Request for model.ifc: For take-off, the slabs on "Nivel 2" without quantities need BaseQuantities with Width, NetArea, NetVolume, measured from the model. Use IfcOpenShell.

First a look at what the model holds.

```python
import ifcopenshell
import ifcopenshell.util.element
import ifcopenshell.util.unit

model = ifcopenshell.open("model.ifc")
print(model.schema)
for unit_type in ("LENGTHUNIT", "AREAUNIT", "VOLUMEUNIT"):
    print(unit_type, ifcopenshell.util.unit.calculate_unit_scale(model, unit_type))
storey = next(s for s in model.by_type("IfcBuildingStorey") if s.Name == "Nivel 2")
slabs = [e for e in ifcopenshell.util.element.get_decomposition(storey) if e.is_a("IfcSlab")]
for e in sorted(slabs, key=lambda e: e.id()):
    print(e.id(), e.is_a(), e.Name, list(ifcopenshell.util.element.get_psets(e, qtos_only=True)), sep=" | ")
```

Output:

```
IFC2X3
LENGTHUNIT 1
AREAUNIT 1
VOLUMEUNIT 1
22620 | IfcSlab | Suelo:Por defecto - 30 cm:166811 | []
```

```python
import ifcopenshell
import ifcopenshell.api.pset
import ifcopenshell.geom
import ifcopenshell.util.element
import ifcopenshell.util.shape
import ifcopenshell.util.unit

model = ifcopenshell.open("model.ifc")
unit_scale = ifcopenshell.util.unit.calculate_unit_scale(model)
area_scale = ifcopenshell.util.unit.calculate_unit_scale(model, "AREAUNIT")
volume_scale = ifcopenshell.util.unit.calculate_unit_scale(model, "VOLUMEUNIT")
settings = ifcopenshell.geom.settings()

storey = next(s for s in model.by_type("IfcBuildingStorey") if s.Name == "Nivel 2")
slabs = [e for e in ifcopenshell.util.element.get_decomposition(storey) if e.is_a("IfcSlab")]

for e in sorted(slabs, key=lambda e: e.id()):
    if ifcopenshell.util.element.get_psets(e, qtos_only=True, should_inherit=False):
        continue
    # Geometry comes back in metres, in the element's own axes.
    shape = ifcopenshell.geom.create_shape(settings, e)
    values = {
        "Width": ifcopenshell.util.shape.get_z(shape.geometry) / unit_scale,
        "NetArea": ifcopenshell.util.shape.get_footprint_area(shape.geometry) / area_scale,
        "NetVolume": ifcopenshell.util.shape.get_volume(shape.geometry) / volume_scale,
    }
    qto = ifcopenshell.api.pset.add_qto(model, product=e, name="BaseQuantities")
    ifcopenshell.api.pset.edit_qto(model, qto=qto, properties=values)
    print(e.id(), {k: round(v, 3) for k, v in values.items()})

model.write("model-out.ifc")
```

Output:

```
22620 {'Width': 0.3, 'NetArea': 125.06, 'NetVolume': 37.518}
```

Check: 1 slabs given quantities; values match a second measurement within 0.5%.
